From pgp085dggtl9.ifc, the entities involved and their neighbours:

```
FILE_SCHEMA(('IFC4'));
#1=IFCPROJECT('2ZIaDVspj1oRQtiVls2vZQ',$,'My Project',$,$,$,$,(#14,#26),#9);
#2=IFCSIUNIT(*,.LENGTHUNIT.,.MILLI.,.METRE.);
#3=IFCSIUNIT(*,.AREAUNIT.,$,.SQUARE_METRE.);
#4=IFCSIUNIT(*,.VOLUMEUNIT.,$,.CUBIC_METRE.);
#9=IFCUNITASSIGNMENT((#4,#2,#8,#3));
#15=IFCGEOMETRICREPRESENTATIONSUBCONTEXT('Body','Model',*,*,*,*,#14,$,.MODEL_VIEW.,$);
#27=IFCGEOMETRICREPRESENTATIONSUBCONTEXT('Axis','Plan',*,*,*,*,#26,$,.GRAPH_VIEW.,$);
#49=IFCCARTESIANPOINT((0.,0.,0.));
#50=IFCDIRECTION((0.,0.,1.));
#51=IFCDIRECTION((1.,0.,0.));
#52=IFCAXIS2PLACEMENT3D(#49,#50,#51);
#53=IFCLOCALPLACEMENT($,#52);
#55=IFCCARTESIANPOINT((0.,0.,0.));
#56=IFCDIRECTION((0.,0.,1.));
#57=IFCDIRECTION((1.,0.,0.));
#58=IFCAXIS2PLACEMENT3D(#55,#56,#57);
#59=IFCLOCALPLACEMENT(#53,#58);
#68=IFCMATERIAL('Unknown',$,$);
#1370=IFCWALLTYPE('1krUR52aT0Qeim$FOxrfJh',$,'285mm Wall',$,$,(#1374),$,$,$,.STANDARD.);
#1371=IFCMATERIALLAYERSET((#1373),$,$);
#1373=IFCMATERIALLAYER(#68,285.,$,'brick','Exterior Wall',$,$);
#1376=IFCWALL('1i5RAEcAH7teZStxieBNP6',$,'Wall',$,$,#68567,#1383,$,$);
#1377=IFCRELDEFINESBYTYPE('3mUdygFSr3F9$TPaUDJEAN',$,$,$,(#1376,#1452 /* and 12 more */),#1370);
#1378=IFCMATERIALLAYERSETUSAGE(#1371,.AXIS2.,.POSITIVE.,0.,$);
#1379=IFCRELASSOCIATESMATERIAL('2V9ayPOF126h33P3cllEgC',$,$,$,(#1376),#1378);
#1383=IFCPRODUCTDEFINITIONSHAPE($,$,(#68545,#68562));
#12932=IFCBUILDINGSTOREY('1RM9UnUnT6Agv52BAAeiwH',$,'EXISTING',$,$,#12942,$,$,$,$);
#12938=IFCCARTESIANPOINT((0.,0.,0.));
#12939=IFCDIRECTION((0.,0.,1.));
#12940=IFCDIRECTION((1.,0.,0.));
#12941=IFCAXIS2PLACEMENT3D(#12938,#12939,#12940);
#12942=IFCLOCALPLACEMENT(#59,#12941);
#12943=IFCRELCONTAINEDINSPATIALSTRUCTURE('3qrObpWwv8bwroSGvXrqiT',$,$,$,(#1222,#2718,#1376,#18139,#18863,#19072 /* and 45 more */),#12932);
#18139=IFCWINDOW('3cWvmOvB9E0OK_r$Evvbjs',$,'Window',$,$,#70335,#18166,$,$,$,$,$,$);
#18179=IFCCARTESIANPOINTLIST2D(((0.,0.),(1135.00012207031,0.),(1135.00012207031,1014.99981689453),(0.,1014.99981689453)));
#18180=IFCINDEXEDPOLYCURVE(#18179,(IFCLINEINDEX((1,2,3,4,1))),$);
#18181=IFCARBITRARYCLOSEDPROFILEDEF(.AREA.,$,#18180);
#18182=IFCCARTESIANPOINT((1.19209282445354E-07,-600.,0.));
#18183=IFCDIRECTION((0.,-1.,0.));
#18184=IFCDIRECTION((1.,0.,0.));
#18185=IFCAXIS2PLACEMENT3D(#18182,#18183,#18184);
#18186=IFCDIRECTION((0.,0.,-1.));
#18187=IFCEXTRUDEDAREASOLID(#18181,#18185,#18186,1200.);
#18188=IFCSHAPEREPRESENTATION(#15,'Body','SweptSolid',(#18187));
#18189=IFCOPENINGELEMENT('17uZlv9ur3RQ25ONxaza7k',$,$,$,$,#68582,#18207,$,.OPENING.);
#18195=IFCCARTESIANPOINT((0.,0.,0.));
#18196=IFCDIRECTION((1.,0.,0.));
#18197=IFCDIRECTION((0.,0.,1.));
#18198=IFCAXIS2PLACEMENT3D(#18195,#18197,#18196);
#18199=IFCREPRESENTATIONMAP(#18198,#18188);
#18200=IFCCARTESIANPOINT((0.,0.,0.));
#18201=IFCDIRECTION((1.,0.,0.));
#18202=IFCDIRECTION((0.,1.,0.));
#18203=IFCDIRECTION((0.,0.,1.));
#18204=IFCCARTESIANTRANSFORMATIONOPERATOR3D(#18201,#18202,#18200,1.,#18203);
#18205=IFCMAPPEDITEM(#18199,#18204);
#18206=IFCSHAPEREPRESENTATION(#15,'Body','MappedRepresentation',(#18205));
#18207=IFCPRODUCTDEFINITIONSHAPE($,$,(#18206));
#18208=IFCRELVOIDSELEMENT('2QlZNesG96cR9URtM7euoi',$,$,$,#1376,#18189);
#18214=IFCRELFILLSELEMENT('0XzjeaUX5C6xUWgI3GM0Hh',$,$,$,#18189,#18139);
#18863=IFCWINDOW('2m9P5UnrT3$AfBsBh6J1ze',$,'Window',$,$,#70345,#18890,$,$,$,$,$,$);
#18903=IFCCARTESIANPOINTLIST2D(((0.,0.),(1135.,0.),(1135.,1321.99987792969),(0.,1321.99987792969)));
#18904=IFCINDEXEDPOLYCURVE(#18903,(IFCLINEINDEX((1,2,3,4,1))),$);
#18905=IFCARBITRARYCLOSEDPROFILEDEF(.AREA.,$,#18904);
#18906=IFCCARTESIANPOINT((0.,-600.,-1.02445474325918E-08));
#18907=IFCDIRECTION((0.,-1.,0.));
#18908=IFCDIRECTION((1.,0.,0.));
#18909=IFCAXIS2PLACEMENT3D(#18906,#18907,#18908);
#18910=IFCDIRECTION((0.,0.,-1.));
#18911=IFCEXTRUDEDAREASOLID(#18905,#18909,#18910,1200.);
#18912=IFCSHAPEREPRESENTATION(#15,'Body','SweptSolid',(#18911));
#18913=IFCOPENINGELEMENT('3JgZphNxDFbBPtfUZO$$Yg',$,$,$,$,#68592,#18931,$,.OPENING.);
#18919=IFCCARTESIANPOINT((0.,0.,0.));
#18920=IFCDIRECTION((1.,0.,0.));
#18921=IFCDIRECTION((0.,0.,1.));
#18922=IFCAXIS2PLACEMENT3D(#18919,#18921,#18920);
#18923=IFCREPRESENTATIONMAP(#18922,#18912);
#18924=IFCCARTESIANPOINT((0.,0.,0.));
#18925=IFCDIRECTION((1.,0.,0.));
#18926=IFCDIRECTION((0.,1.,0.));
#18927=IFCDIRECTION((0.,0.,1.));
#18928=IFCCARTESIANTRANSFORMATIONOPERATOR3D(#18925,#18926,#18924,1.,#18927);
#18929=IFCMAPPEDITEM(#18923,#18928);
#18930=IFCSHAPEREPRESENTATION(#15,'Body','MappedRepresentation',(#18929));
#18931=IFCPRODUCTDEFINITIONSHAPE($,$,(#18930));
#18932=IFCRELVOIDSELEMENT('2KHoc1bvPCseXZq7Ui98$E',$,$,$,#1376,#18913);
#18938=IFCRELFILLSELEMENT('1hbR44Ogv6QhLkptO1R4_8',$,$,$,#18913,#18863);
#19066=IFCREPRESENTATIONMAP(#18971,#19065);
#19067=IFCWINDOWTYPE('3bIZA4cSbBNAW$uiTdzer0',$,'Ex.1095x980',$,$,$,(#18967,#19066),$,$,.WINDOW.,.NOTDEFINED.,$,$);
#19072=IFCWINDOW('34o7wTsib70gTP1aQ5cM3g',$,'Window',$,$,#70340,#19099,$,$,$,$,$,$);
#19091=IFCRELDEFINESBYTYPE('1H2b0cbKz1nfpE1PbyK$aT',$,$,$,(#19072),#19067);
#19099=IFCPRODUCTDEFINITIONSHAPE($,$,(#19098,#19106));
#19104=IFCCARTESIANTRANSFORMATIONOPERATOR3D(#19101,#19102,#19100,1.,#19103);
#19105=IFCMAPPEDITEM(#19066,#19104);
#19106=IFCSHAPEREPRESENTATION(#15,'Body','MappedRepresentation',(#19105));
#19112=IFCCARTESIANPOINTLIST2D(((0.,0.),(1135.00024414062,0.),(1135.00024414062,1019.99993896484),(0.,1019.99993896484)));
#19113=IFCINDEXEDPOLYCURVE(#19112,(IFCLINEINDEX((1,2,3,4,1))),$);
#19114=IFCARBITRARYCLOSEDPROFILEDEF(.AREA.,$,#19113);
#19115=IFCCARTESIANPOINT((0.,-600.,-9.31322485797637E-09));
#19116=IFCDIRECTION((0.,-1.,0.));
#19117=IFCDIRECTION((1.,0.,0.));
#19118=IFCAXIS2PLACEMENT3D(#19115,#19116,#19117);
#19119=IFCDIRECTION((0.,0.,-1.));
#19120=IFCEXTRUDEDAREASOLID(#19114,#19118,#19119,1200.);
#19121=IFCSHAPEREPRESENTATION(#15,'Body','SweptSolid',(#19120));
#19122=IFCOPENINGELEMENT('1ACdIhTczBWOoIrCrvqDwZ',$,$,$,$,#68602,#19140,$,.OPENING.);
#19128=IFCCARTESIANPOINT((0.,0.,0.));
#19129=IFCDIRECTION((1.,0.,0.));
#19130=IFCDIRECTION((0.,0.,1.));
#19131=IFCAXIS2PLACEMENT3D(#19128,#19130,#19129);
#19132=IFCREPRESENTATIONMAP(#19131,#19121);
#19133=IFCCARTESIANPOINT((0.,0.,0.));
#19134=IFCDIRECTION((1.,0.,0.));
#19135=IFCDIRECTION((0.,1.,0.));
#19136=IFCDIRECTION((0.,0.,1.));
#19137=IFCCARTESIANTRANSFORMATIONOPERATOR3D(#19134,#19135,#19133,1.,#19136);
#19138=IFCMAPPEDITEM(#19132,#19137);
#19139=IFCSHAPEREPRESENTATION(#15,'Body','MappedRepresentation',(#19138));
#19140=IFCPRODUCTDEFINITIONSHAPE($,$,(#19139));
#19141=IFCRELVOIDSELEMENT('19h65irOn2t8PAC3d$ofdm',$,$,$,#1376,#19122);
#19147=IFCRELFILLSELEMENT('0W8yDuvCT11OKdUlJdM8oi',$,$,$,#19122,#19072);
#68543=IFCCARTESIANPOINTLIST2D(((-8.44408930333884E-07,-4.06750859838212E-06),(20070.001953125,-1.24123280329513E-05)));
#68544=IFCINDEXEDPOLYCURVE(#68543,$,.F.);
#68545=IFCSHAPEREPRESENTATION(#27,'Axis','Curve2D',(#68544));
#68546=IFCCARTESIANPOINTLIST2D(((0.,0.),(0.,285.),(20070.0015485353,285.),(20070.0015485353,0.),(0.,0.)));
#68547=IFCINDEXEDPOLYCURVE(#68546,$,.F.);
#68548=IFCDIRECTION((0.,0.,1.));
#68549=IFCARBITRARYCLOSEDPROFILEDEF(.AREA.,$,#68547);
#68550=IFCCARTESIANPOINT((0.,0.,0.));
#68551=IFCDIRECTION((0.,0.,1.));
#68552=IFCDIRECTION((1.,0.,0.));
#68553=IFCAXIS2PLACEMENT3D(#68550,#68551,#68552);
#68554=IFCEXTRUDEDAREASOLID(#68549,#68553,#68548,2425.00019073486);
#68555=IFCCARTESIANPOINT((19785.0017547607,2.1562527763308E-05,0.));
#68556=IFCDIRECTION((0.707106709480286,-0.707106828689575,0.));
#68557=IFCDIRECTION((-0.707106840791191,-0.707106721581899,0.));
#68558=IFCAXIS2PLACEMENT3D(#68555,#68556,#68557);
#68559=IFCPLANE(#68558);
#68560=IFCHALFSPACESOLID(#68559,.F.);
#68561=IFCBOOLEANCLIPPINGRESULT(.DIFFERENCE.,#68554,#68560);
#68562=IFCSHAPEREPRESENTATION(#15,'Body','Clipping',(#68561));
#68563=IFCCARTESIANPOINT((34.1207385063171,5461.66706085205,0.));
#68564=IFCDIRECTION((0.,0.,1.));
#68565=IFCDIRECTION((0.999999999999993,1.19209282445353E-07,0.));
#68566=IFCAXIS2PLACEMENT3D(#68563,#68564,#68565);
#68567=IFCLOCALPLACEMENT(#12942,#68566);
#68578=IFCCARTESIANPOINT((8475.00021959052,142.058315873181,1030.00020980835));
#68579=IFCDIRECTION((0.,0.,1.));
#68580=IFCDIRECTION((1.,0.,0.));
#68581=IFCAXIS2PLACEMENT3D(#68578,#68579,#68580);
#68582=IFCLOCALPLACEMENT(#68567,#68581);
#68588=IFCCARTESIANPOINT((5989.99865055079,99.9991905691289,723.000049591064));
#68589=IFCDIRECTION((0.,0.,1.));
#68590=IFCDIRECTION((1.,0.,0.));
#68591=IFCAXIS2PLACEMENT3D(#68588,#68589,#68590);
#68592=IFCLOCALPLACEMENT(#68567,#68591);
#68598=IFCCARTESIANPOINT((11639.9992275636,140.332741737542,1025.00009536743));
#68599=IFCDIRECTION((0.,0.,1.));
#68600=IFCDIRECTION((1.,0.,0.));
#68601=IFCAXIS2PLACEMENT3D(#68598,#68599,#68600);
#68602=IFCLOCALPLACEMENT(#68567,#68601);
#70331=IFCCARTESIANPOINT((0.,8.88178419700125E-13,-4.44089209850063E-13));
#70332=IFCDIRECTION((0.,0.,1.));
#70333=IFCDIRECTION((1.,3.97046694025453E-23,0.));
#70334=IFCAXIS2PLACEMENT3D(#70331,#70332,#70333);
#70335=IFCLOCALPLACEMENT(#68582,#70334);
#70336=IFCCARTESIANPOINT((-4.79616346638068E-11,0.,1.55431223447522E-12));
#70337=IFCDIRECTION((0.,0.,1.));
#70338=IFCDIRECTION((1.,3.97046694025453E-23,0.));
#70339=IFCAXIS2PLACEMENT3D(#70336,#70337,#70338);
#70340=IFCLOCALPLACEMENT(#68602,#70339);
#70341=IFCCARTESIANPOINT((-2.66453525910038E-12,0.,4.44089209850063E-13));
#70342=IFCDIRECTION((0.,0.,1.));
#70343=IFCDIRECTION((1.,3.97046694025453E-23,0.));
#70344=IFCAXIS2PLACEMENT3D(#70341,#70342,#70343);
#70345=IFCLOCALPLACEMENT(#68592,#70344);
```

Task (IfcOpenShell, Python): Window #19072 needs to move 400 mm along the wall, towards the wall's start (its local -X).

```python
import ifcopenshell
import ifcopenshell.api.geometry
import ifcopenshell.util.placement
import ifcopenshell.util.unit

model = ifcopenshell.open("pgp085dggtl9.ifc")
unit_scale = ifcopenshell.util.unit.calculate_unit_scale(model)

window = model.by_id(19072)
opening = window.FillsVoids[0].RelatingOpeningElement
wall = opening.VoidsElements[0].RelatingBuildingElement

wall_matrix = ifcopenshell.util.placement.get_local_placement(wall.ObjectPlacement)
shift = wall_matrix[:3, 0] * -0.4 / unit_scale
before = ifcopenshell.util.placement.get_local_placement(window.ObjectPlacement)[:3, 3].copy()

# The window is placed relative to its opening, so it follows when the opening moves.
matrix = ifcopenshell.util.placement.get_local_placement(opening.ObjectPlacement)
matrix[:3, 3] += shift
ifcopenshell.api.geometry.edit_object_placement(
    model, product=opening, matrix=matrix, is_si=False, should_transform_children=True
)

after = ifcopenshell.util.placement.get_local_placement(window.ObjectPlacement)[:3, 3]
print("window moved by", (after - before).round(3) + 0.0)

model.write("pgp085dggtl9_updated.ifc")
```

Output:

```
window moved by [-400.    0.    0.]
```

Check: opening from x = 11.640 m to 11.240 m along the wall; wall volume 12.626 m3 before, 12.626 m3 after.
